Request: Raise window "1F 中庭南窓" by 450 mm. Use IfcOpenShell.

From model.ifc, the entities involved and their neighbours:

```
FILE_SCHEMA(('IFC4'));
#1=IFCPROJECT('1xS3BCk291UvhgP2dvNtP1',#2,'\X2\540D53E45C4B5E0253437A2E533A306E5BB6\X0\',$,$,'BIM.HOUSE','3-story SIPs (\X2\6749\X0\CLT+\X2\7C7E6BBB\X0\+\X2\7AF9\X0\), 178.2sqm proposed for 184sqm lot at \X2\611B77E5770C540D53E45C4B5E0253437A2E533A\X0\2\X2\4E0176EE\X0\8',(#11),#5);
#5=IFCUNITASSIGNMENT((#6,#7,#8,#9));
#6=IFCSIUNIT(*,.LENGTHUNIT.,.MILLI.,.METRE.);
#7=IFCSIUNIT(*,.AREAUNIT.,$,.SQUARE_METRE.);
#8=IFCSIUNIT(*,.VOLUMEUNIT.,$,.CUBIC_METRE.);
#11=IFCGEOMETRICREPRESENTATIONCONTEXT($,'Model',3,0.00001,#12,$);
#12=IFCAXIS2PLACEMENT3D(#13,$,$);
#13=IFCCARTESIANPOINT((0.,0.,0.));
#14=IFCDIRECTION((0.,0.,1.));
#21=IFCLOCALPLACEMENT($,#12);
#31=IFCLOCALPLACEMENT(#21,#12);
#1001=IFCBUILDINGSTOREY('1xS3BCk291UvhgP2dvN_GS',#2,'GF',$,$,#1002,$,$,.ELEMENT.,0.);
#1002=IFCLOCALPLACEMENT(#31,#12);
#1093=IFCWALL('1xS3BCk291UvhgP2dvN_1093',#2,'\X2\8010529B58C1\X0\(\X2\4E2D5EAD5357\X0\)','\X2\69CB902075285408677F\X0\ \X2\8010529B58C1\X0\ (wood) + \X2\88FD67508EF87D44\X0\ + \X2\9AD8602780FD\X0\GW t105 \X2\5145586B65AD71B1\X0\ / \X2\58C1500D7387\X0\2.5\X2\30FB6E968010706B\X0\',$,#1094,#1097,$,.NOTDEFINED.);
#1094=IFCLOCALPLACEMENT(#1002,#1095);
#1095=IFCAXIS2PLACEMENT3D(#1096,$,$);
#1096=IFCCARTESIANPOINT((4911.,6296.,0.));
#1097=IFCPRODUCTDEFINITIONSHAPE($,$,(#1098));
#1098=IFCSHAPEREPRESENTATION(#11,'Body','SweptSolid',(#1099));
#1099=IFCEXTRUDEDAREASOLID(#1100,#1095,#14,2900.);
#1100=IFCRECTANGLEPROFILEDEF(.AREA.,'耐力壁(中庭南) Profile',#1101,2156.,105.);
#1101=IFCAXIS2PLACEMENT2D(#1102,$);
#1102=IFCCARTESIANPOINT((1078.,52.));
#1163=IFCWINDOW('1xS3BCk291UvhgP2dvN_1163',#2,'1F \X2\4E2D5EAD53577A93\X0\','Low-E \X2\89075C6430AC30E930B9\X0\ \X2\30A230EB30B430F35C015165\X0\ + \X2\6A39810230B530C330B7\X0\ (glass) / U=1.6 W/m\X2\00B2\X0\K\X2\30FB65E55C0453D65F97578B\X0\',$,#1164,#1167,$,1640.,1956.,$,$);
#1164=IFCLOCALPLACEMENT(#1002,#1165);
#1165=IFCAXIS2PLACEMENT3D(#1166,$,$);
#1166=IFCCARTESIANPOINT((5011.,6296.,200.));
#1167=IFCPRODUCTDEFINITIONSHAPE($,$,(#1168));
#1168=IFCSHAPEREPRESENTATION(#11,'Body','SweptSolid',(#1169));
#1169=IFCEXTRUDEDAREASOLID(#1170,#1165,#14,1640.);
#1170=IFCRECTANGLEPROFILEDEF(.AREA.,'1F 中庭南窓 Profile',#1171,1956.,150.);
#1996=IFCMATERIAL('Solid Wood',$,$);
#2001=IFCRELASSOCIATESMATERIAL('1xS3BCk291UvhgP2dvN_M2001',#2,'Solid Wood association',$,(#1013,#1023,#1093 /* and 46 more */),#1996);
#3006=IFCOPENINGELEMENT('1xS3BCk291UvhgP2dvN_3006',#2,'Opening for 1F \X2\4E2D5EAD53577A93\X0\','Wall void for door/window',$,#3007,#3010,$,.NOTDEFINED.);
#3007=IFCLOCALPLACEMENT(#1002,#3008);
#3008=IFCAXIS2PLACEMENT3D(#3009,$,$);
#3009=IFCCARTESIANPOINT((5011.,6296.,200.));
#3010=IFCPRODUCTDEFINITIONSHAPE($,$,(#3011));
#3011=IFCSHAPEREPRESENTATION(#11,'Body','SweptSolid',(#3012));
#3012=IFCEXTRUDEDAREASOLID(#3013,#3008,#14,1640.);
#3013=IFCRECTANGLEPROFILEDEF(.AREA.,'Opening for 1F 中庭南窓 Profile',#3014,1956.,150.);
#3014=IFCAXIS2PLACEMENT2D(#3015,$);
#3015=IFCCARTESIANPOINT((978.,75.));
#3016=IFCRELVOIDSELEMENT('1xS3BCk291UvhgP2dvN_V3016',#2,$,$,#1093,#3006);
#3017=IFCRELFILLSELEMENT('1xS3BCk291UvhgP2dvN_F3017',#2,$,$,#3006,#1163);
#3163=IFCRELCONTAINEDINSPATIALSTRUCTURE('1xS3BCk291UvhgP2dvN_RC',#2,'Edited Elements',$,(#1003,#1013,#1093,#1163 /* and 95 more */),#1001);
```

```python
import numpy as np
import ifcopenshell
import ifcopenshell.api.geometry
import ifcopenshell.util.placement
import ifcopenshell.util.unit

model = ifcopenshell.open("model.ifc")
unit_scale = ifcopenshell.util.unit.calculate_unit_scale(model)

window = model.by_guid("1xS3BCk291UvhgP2dvN_1163")
opening = window.FillsVoids[0].RelatingOpeningElement
dz = 0.45 / unit_scale

shift = np.array([0.0, 0.0, dz])
# The window is not placed relative to its opening, so move both.
for product in (opening, window):
    matrix = ifcopenshell.util.placement.get_local_placement(product.ObjectPlacement)
    matrix[:3, 3] += shift
    ifcopenshell.api.geometry.edit_object_placement(model, product=product, matrix=matrix, is_si=False)

print(f"moved by {dz * unit_scale:+.3f} m")

model.write("model_rev.ifc")
```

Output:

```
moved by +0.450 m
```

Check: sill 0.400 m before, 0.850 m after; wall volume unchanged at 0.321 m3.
